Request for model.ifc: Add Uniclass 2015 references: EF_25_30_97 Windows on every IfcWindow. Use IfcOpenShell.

First a look at what the model holds.

```python
import ifcopenshell

model = ifcopenshell.open("model.ifc")
print(model.schema)
print("classifications:", [c.Name for c in model.by_type("IfcClassification")])
for ifc_class in ("IfcDoor", "IfcRoof", "IfcStair", "IfcWall", "IfcWindow"):
    print(ifc_class, len(model.by_type(ifc_class)))
```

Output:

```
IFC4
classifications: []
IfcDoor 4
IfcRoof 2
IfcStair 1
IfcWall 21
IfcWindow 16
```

```python
import ifcopenshell
import ifcopenshell.api.classification

model = ifcopenshell.open("model.ifc")

system = ifcopenshell.api.classification.add_classification(model, classification="Uniclass 2015")

codes = {
    "IfcWindow": ("EF_25_30_97", "Windows"),
}
for ifc_class, (code, name) in codes.items():
    products = model.by_type(ifc_class)
    ifcopenshell.api.classification.add_reference(
        model, products=products, classification=system, identification=code, name=name
    )
    print(code, len(products))

model.write("model_rev.ifc")
```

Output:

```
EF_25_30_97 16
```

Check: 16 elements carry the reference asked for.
